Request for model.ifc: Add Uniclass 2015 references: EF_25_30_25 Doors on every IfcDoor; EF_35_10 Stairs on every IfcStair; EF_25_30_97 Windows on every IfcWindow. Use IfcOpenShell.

First a look at what the model holds.

```python
import ifcopenshell

model = ifcopenshell.open("model.ifc")
print(model.schema)
print("classifications:", [c.Name for c in model.by_type("IfcClassification")])
for ifc_class in ("IfcDoor", "IfcRoof", "IfcStair", "IfcWall", "IfcWindow"):
    print(ifc_class, len(model.by_type(ifc_class)))
```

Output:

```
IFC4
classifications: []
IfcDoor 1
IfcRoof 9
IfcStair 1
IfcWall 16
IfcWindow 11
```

```python
import ifcopenshell
import ifcopenshell.api.classification

model = ifcopenshell.open("model.ifc")

system = ifcopenshell.api.classification.add_classification(model, classification="Uniclass 2015")

codes = {
    "IfcDoor": ("EF_25_30_25", "Doors"),
    "IfcStair": ("EF_35_10", "Stairs"),
    "IfcWindow": ("EF_25_30_97", "Windows"),
}
for ifc_class, (code, name) in codes.items():
    products = model.by_type(ifc_class)
    ifcopenshell.api.classification.add_reference(
        model, products=products, classification=system, identification=code, name=name
    )
    print(code, len(products))

model.write("model_edited.ifc")
```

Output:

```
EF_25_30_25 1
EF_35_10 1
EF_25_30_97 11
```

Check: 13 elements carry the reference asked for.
